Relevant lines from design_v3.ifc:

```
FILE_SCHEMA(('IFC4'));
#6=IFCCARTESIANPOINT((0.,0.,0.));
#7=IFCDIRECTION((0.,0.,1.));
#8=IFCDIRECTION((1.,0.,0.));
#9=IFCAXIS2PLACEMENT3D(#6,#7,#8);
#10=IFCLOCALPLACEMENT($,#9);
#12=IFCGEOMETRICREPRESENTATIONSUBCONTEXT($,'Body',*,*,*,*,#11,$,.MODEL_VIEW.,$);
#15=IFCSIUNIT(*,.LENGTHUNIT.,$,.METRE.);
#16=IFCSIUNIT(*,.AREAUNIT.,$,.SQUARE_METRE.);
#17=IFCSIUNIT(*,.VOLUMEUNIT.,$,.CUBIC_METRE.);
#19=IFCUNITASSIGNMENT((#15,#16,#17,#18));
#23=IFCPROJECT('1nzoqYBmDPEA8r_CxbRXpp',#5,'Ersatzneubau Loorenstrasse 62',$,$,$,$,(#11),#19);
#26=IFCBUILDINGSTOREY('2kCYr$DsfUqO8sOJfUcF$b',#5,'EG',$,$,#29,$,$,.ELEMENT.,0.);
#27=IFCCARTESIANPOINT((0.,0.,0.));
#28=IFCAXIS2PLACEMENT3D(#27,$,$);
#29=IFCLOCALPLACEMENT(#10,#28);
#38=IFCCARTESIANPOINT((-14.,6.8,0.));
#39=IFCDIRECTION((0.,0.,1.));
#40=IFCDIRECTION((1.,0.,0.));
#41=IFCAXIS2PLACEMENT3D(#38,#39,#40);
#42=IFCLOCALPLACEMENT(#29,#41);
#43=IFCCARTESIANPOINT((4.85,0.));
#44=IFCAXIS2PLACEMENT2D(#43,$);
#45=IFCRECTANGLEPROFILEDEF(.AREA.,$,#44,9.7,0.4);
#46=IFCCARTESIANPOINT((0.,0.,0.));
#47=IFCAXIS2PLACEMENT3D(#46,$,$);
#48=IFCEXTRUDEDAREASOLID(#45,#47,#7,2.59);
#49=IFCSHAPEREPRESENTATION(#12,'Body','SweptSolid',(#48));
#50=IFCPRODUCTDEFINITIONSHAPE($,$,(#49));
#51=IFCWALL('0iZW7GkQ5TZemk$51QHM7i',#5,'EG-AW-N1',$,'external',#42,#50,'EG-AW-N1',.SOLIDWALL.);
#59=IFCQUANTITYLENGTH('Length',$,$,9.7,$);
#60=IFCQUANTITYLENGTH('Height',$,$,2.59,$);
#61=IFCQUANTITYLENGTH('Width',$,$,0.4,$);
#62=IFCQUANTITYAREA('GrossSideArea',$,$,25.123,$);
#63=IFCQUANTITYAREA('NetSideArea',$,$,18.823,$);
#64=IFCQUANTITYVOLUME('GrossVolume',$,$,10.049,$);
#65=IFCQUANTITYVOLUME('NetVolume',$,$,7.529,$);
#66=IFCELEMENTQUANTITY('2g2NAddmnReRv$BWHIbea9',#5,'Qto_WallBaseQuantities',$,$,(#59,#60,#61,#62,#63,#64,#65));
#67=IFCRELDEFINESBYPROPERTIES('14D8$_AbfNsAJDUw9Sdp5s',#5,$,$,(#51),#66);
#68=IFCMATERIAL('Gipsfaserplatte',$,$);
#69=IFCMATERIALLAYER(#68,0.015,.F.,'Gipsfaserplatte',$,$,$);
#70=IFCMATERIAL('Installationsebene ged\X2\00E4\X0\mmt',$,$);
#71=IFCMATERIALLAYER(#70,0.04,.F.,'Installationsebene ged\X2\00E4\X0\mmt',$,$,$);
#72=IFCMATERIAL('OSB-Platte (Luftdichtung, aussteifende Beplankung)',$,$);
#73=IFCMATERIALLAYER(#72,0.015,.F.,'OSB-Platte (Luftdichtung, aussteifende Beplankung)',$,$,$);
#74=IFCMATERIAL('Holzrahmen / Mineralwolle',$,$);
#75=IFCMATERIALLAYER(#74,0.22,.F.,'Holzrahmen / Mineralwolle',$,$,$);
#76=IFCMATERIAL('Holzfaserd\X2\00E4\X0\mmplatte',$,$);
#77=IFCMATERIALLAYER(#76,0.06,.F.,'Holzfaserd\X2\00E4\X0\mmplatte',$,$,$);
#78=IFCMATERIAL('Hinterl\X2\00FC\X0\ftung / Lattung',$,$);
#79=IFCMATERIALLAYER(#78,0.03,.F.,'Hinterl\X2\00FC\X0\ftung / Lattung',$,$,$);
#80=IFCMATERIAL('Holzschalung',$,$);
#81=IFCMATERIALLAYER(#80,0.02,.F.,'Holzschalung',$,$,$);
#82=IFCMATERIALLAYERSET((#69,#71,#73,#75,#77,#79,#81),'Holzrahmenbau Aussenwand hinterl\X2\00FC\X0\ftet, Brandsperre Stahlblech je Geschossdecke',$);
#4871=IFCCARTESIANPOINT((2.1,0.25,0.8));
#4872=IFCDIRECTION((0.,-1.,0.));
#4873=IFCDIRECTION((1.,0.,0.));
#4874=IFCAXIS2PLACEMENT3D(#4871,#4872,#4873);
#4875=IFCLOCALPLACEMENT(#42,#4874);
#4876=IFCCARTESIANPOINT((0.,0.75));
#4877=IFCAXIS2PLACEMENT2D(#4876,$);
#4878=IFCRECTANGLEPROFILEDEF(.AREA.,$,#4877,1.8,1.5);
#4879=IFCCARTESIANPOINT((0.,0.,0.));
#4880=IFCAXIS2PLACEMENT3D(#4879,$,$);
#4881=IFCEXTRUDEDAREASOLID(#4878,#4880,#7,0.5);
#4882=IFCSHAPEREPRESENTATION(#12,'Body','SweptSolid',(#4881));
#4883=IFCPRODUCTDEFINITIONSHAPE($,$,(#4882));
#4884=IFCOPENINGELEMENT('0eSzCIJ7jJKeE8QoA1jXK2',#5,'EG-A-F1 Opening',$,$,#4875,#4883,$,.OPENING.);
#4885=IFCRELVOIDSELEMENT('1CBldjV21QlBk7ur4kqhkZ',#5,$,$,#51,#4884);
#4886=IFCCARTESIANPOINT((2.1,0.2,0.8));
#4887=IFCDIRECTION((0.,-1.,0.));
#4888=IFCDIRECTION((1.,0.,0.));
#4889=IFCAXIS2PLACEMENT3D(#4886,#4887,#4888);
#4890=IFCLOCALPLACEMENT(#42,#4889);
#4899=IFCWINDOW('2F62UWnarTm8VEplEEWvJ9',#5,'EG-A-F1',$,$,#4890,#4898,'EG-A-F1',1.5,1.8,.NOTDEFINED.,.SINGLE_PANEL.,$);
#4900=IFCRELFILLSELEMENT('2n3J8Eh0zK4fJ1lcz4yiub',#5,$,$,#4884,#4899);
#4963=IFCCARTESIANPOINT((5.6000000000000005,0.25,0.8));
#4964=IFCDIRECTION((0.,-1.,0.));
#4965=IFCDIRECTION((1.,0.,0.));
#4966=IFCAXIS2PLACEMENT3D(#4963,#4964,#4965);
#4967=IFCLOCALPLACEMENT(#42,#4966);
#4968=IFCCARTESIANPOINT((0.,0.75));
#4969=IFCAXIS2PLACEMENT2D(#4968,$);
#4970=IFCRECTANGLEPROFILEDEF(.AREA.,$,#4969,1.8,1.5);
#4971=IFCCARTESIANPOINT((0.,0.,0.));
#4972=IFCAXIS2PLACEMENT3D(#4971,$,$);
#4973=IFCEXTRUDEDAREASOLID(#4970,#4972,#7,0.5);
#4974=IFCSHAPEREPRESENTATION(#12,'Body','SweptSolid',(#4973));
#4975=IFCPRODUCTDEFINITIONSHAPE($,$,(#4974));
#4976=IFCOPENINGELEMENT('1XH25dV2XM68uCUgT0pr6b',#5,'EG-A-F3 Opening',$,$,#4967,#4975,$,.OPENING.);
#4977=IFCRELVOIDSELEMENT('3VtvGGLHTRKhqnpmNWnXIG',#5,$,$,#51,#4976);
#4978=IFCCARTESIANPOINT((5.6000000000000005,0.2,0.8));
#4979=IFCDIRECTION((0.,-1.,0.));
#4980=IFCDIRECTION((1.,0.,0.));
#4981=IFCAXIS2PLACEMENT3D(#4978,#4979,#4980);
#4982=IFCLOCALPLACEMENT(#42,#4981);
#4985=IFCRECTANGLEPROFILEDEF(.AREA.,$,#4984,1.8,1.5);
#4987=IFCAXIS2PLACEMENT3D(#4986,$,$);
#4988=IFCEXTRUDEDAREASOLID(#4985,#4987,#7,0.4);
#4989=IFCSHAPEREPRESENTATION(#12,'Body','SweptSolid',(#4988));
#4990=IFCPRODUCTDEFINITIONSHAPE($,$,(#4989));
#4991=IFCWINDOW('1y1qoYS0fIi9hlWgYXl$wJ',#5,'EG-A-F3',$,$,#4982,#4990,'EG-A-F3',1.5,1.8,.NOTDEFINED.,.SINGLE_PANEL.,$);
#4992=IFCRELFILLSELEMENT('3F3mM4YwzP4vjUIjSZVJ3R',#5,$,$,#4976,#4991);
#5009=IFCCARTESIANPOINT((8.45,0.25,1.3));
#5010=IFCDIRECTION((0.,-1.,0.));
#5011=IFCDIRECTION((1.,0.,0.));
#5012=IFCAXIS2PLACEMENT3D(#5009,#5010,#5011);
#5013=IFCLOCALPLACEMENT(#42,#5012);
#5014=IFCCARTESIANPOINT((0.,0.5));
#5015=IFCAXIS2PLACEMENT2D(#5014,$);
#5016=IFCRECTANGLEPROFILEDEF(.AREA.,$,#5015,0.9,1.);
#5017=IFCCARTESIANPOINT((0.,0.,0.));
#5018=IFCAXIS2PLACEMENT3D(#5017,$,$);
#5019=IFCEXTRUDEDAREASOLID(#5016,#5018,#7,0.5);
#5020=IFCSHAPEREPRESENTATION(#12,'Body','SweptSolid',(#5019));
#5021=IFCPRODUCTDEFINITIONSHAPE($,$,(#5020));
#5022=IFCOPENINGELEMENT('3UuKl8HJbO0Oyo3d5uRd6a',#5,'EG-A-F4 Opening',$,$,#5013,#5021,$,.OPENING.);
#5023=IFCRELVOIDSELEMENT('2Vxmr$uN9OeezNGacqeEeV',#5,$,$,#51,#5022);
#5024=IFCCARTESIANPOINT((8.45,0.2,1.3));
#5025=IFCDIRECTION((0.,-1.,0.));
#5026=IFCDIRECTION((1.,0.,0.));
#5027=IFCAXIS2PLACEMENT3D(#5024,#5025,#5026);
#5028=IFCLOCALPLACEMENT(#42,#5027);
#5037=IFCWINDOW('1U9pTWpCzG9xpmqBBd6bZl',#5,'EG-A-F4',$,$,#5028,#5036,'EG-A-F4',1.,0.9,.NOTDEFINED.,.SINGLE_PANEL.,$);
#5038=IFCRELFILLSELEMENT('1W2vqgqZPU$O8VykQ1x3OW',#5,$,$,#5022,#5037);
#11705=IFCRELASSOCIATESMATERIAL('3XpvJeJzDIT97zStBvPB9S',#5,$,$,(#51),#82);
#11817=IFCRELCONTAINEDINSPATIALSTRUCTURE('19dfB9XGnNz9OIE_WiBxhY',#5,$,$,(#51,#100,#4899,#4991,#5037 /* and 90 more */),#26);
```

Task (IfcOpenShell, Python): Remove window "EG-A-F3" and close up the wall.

```python
import ifcopenshell
import ifcopenshell.api.feature
import ifcopenshell.api.pset
import ifcopenshell.api.root
import ifcopenshell.geom
import ifcopenshell.util.element
import ifcopenshell.util.shape
import ifcopenshell.util.unit

model = ifcopenshell.open("design_v3.ifc")
area_scale = ifcopenshell.util.unit.calculate_unit_scale(model, "AREAUNIT")
volume_scale = ifcopenshell.util.unit.calculate_unit_scale(model, "VOLUMEUNIT")
settings = ifcopenshell.geom.settings()


def volume(element):
    """Net volume in cubic metres, openings subtracted."""
    shape = ifcopenshell.geom.create_shape(settings, element)
    return ifcopenshell.util.shape.get_volume(shape.geometry)


window = model.by_id(4991)
opening = window.FillsVoids[0].RelatingOpeningElement
wall = opening.VoidsElements[0].RelatingBuildingElement
before = volume(wall)

ifcopenshell.api.root.remove_product(model, product=window)
ifcopenshell.api.feature.remove_feature(model, feature=opening)

after = volume(wall)
thickness = 0.4  # wall thickness in metres

# Update the wall's stored quantities.
qto = model.by_id(ifcopenshell.util.element.get_pset(wall, "Qto_WallBaseQuantities", should_inherit=False)["id"])
ifcopenshell.api.pset.edit_qto(model, qto=qto, properties={
    "NetSideArea": after / thickness / area_scale,
    "NetVolume": after / volume_scale,
})

print(f"wall volume {before:.3f} -> {after:.3f} m3")

model.write("design_v3_rev.ifc")
```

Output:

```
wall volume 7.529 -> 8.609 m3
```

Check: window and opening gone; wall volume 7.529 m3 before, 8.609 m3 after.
